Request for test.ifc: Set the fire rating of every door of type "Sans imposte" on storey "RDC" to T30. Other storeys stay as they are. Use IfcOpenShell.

First a look at what the model holds.

```python
import ifcopenshell
import ifcopenshell.util.element

model = ifcopenshell.open("test.ifc")
print(model.schema)
storey = next(s for s in model.by_type("IfcBuildingStorey") if s.Name == "RDC")
doors = [e for e in ifcopenshell.util.element.get_decomposition(storey) if e.is_a("IfcDoor")]
seen = {}
for e in doors:
    element_type = ifcopenshell.util.element.get_type(e)
    key = (element_type.Name if element_type != e and element_type else None, ifcopenshell.util.element.get_pset(e, "Pset_DoorCommon", "FireRating"))
    seen[key] = seen.get(key, 0) + 1
for (name, value), count in sorted(seen.items(), key=str):
    print(count, "x", name, "|", value)
```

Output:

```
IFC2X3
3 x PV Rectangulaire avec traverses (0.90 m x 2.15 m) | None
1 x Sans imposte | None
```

```python
import ifcopenshell
import ifcopenshell.api.pset
import ifcopenshell.util.element

model = ifcopenshell.open("test.ifc")

storey = next(s for s in model.by_type("IfcBuildingStorey") if s.Name == "RDC")
doors = [e for e in ifcopenshell.util.element.get_decomposition(storey) if e.is_a("IfcDoor")]

count = 0
for e in doors:
    element_type = ifcopenshell.util.element.get_type(e)
    if element_type in (None, e) or element_type.Name != "Sans imposte":
        continue
    # add_pset returns the element's existing set when there is one.
    pset = ifcopenshell.api.pset.add_pset(model, product=e, name="Pset_DoorCommon")
    ifcopenshell.api.pset.edit_pset(model, pset=pset, properties={"FireRating": "T30"})
    count += 1

print(count, "doors updated")

model.write("test_updated.ifc")
```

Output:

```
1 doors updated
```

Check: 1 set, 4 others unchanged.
